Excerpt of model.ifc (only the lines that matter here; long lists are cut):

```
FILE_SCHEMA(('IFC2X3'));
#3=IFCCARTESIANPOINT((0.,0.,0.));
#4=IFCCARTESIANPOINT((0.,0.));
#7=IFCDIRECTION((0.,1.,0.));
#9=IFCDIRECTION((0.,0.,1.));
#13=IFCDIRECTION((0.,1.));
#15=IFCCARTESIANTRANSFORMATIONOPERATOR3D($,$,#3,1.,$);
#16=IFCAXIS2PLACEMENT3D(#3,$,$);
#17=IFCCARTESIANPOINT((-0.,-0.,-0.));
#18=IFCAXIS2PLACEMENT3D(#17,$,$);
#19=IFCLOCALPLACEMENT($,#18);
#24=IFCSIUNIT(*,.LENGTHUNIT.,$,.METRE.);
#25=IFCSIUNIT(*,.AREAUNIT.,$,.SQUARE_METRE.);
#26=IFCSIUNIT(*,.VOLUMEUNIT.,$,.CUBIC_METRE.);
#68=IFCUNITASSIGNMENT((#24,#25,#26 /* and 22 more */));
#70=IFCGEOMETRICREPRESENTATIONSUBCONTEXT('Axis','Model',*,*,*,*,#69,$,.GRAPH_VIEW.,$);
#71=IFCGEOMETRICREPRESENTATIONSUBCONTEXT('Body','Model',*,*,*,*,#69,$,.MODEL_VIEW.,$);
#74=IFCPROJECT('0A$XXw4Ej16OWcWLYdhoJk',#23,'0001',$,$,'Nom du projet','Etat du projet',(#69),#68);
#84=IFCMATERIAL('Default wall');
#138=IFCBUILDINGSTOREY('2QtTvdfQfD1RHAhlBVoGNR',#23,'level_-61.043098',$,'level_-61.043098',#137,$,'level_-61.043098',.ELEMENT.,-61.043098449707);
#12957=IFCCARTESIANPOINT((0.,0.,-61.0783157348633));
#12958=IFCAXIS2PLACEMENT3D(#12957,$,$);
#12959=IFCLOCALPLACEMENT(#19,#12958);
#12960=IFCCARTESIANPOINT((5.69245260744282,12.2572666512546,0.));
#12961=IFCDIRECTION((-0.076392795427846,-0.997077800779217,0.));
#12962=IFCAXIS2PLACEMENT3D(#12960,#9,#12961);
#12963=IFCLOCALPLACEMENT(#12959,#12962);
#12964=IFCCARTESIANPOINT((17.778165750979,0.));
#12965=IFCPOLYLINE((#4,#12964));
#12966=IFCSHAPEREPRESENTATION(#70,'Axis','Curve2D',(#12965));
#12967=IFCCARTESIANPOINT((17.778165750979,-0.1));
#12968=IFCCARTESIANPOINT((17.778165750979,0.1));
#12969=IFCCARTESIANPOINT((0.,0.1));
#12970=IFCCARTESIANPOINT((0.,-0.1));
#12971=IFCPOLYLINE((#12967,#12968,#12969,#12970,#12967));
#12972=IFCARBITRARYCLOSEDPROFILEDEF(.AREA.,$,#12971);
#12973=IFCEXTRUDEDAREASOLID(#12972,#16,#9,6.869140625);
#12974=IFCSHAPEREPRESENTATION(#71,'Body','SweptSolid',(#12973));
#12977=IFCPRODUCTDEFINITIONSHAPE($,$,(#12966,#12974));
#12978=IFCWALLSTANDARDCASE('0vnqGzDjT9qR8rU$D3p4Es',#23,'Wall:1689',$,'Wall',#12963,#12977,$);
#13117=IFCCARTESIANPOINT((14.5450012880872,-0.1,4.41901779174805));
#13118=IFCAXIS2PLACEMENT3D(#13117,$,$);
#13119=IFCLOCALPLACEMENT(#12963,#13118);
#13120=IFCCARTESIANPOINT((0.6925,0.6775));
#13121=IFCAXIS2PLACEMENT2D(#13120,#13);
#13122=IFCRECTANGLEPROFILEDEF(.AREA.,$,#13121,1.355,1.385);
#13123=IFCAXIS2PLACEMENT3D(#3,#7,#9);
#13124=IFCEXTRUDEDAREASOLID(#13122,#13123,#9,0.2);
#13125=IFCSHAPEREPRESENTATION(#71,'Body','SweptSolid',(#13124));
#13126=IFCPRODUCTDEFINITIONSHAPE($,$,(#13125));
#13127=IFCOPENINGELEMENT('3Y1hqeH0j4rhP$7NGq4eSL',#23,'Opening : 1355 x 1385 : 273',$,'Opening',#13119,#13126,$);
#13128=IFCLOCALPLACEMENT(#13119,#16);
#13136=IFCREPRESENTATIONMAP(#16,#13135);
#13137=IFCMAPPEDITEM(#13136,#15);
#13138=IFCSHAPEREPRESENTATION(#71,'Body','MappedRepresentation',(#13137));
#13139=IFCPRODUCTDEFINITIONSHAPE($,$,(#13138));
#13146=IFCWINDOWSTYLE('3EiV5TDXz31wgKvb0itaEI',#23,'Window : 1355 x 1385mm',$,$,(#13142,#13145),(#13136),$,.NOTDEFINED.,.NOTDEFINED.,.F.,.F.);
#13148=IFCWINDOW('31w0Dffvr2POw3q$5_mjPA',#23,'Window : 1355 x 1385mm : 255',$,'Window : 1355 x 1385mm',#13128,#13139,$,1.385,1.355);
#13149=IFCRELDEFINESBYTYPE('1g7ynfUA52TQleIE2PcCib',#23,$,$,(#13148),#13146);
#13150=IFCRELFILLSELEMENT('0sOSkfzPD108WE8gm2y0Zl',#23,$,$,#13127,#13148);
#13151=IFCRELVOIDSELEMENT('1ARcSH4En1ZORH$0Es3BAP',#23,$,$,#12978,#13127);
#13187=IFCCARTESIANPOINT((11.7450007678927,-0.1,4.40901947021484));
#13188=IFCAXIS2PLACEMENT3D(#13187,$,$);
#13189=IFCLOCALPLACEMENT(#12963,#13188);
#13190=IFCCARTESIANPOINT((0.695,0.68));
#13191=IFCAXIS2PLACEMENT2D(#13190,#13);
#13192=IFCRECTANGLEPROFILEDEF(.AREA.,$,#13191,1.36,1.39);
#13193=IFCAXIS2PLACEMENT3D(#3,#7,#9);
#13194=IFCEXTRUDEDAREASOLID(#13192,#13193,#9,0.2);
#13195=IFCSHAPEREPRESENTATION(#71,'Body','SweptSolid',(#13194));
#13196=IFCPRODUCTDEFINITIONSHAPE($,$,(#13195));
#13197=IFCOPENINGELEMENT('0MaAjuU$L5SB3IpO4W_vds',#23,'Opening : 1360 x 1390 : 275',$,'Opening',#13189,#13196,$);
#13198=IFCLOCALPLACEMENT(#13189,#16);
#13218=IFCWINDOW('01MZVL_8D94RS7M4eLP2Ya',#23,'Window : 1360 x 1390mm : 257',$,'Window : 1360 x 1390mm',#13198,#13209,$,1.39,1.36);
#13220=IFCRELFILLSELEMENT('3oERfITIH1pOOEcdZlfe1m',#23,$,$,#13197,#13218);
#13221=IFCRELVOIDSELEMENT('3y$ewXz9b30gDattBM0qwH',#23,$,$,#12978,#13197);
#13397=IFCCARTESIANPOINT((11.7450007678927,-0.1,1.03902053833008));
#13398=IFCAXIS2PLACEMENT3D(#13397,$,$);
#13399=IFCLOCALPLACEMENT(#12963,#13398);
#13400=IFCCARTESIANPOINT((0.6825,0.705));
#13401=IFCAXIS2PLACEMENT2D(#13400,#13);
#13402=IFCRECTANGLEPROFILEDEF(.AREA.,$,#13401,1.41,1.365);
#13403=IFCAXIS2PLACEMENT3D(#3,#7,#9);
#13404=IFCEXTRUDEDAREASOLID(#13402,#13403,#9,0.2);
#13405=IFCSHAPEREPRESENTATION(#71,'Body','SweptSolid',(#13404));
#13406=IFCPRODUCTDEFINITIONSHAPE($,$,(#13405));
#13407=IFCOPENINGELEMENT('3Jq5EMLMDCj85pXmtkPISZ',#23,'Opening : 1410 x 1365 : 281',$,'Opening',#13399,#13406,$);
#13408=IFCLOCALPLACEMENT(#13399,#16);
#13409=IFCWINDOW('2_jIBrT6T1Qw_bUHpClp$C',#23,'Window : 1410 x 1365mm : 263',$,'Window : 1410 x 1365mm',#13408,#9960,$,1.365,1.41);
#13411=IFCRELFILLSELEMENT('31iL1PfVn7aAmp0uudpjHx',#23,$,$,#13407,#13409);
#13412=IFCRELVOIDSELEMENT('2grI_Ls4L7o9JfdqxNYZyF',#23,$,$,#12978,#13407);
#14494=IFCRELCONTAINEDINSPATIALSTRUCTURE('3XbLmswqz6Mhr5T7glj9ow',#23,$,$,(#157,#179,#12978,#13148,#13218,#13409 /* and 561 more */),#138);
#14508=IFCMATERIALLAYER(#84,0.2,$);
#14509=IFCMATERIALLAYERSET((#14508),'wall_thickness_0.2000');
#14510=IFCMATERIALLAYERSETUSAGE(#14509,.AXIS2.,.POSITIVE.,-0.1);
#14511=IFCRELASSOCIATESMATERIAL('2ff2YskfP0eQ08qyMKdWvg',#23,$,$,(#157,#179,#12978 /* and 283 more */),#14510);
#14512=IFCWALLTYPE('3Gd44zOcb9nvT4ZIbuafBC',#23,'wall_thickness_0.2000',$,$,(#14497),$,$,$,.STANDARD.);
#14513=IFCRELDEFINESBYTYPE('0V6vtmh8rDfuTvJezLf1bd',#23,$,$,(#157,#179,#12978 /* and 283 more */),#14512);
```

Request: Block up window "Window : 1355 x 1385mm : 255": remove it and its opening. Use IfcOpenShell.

```python
import ifcopenshell
import ifcopenshell.api.feature
import ifcopenshell.api.root
import ifcopenshell.geom
import ifcopenshell.util.shape

model = ifcopenshell.open("model.ifc")
settings = ifcopenshell.geom.settings()


def volume(element):
    """Net volume in cubic metres, openings subtracted."""
    shape = ifcopenshell.geom.create_shape(settings, element)
    return ifcopenshell.util.shape.get_volume(shape.geometry)


window = model.by_guid("31w0Dffvr2POw3q$5_mjPA")
opening = window.FillsVoids[0].RelatingOpeningElement
wall = opening.VoidsElements[0].RelatingBuildingElement
before = volume(wall)

ifcopenshell.api.root.remove_product(model, product=window)
ifcopenshell.api.feature.remove_feature(model, feature=opening)

after = volume(wall)

print(f"wall volume {before:.3f} -> {after:.3f} m3")

model.write("model_rev.ifc")
```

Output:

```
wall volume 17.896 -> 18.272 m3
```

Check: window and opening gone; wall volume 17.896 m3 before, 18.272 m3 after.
